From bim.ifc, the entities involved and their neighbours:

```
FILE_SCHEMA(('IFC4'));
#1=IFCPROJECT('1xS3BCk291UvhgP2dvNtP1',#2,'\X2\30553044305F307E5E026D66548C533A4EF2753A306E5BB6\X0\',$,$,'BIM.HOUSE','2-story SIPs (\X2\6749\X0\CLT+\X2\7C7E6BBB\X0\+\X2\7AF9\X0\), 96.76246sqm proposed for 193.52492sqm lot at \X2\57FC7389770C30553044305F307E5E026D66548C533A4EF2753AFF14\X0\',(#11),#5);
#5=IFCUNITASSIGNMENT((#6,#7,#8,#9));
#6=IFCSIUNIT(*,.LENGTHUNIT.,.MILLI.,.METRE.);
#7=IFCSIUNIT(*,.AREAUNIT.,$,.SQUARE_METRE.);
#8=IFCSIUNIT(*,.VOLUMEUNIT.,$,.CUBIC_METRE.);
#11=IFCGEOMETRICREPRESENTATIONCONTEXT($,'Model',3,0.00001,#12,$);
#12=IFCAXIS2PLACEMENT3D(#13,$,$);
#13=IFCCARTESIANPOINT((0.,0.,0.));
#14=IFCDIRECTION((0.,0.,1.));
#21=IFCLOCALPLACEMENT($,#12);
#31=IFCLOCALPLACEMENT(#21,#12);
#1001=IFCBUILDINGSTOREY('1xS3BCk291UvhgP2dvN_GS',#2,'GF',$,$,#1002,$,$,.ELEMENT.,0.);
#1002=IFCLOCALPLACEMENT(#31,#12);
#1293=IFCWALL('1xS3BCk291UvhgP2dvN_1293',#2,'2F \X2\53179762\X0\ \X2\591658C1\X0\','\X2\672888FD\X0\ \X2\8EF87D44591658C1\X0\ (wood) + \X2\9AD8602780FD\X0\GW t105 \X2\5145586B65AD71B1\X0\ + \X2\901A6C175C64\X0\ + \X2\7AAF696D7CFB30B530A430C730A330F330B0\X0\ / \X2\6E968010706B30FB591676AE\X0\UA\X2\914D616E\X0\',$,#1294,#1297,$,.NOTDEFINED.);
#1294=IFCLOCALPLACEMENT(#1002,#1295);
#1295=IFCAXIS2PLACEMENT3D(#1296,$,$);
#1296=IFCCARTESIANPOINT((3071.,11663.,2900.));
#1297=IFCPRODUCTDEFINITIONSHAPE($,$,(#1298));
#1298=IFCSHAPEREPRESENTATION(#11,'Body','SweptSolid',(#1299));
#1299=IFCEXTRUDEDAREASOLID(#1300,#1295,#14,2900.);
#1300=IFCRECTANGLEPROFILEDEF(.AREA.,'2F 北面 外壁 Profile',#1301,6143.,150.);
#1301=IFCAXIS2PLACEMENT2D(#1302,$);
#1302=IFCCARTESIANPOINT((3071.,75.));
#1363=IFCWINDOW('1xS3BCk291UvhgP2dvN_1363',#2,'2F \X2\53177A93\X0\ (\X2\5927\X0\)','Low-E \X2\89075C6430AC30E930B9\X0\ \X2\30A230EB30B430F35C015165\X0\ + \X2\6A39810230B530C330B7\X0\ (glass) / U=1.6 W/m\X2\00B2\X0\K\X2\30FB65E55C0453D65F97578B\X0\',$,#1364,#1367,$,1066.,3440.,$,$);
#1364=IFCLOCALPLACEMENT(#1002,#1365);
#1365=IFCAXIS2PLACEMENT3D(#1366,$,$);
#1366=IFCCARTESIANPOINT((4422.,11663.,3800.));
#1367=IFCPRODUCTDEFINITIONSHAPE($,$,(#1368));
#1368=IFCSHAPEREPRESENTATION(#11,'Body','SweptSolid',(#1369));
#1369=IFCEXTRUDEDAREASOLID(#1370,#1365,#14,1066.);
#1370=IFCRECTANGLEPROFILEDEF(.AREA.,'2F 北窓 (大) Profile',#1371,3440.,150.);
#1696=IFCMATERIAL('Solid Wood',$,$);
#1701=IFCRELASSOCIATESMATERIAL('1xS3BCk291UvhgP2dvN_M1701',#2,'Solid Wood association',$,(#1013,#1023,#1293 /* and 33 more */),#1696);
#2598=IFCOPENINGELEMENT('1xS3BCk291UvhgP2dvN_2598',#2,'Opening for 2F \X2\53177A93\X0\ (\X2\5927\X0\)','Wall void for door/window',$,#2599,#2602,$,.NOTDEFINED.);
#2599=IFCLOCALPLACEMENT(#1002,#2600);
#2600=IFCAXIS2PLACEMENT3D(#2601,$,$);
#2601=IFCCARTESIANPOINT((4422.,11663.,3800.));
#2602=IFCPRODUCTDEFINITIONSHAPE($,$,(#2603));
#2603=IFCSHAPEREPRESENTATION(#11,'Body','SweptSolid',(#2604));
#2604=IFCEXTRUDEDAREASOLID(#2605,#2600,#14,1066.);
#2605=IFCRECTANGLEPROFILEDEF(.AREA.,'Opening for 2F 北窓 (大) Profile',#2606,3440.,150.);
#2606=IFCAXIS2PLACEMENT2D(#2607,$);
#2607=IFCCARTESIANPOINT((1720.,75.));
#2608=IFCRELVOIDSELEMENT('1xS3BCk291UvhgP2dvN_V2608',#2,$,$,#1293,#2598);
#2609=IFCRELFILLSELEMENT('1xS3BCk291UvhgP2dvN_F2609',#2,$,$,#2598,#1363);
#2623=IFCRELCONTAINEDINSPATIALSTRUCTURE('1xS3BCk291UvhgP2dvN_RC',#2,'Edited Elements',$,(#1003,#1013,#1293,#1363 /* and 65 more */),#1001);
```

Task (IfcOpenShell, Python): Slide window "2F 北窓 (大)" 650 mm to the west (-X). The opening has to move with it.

```python
import ifcopenshell
import ifcopenshell.api.geometry
import ifcopenshell.util.placement
import ifcopenshell.util.unit

model = ifcopenshell.open("bim.ifc")
unit_scale = ifcopenshell.util.unit.calculate_unit_scale(model)

window = model.by_guid("1xS3BCk291UvhgP2dvN_1363")
opening = window.FillsVoids[0].RelatingOpeningElement
wall = opening.VoidsElements[0].RelatingBuildingElement

wall_matrix = ifcopenshell.util.placement.get_local_placement(wall.ObjectPlacement)
shift = wall_matrix[:3, 0] * -0.65 / unit_scale
before = ifcopenshell.util.placement.get_local_placement(window.ObjectPlacement)[:3, 3].copy()

# The window is not placed relative to its opening, so move both.
for product in (opening, window):
    matrix = ifcopenshell.util.placement.get_local_placement(product.ObjectPlacement)
    matrix[:3, 3] += shift
    ifcopenshell.api.geometry.edit_object_placement(model, product=product, matrix=matrix, is_si=False)

after = ifcopenshell.util.placement.get_local_placement(window.ObjectPlacement)[:3, 3]
print("window moved by", (after - before).round(3) + 0.0)

model.write("bim_edited.ifc")
```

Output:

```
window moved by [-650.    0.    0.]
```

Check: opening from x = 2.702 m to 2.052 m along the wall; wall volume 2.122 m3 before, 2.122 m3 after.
